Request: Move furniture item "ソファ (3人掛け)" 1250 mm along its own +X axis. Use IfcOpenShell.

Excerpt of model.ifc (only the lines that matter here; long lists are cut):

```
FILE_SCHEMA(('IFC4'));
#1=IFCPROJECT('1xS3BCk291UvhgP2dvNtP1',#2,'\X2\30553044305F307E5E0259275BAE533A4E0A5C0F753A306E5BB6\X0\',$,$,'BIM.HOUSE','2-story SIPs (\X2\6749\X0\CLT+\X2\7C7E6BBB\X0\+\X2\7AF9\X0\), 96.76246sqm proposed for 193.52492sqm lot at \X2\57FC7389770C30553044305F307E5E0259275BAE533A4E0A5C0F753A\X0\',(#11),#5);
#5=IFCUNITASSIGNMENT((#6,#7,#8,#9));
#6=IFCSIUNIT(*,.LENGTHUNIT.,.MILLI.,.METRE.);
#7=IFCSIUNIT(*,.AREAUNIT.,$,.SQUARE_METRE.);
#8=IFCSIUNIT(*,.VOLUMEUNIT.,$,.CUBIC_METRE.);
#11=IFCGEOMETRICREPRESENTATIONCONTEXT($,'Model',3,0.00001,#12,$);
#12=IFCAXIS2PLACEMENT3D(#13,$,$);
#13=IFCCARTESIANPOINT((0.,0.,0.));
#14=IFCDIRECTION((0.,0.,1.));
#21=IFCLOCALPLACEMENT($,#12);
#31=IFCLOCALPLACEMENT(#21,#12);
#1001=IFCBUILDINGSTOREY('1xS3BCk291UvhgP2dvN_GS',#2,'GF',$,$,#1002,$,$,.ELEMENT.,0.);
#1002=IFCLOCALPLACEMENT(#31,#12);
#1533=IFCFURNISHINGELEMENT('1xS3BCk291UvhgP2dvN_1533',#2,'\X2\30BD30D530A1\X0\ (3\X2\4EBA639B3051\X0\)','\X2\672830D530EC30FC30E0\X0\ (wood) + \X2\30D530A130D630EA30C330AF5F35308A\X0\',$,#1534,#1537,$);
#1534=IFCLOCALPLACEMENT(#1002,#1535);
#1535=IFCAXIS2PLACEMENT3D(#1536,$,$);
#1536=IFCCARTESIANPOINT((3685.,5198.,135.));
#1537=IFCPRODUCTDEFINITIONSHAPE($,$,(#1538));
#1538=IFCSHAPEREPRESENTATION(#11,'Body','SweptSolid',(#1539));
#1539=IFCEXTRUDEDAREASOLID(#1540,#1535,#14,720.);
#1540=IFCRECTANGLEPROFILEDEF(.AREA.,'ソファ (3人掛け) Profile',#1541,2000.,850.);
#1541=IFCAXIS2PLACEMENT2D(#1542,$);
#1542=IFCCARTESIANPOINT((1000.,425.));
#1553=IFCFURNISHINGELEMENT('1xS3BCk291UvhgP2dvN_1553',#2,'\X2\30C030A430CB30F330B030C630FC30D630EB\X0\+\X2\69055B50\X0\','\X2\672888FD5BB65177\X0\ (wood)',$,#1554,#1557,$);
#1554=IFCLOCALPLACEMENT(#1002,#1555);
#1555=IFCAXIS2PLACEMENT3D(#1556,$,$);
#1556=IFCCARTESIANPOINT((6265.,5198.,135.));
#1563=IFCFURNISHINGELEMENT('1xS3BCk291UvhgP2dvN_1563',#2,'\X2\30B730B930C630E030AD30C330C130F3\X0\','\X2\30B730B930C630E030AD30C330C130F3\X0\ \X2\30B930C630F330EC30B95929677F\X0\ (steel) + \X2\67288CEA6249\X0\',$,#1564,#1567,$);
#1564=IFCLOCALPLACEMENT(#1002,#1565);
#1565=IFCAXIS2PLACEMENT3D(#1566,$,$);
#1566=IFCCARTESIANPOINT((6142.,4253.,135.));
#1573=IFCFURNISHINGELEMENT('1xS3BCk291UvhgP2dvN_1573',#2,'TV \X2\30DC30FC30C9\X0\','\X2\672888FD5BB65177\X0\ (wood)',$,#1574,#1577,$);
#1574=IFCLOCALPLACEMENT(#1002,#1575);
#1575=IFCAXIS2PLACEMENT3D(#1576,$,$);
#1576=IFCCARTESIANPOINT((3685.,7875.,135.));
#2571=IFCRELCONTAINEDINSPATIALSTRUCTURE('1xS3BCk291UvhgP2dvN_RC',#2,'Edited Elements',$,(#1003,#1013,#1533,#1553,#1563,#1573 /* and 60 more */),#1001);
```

```python
import ifcopenshell
import ifcopenshell.api.geometry
import ifcopenshell.util.placement
import ifcopenshell.util.unit

model = ifcopenshell.open("model.ifc")
unit_scale = ifcopenshell.util.unit.calculate_unit_scale(model)

item = model.by_guid("1xS3BCk291UvhgP2dvN_1533")
matrix = ifcopenshell.util.placement.get_local_placement(item.ObjectPlacement)
matrix[:3, 3] += matrix[:3, 0] * 1.25 / unit_scale
ifcopenshell.api.geometry.edit_object_placement(model, product=item, matrix=matrix, is_si=False)

print(ifcopenshell.util.placement.get_local_placement(item.ObjectPlacement).round(3) + 0.0)

model.write("model_edited.ifc")
```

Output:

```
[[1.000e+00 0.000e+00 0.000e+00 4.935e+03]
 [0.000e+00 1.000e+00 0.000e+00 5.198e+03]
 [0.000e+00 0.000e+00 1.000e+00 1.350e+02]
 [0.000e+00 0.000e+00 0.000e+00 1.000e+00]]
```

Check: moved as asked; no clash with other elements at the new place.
